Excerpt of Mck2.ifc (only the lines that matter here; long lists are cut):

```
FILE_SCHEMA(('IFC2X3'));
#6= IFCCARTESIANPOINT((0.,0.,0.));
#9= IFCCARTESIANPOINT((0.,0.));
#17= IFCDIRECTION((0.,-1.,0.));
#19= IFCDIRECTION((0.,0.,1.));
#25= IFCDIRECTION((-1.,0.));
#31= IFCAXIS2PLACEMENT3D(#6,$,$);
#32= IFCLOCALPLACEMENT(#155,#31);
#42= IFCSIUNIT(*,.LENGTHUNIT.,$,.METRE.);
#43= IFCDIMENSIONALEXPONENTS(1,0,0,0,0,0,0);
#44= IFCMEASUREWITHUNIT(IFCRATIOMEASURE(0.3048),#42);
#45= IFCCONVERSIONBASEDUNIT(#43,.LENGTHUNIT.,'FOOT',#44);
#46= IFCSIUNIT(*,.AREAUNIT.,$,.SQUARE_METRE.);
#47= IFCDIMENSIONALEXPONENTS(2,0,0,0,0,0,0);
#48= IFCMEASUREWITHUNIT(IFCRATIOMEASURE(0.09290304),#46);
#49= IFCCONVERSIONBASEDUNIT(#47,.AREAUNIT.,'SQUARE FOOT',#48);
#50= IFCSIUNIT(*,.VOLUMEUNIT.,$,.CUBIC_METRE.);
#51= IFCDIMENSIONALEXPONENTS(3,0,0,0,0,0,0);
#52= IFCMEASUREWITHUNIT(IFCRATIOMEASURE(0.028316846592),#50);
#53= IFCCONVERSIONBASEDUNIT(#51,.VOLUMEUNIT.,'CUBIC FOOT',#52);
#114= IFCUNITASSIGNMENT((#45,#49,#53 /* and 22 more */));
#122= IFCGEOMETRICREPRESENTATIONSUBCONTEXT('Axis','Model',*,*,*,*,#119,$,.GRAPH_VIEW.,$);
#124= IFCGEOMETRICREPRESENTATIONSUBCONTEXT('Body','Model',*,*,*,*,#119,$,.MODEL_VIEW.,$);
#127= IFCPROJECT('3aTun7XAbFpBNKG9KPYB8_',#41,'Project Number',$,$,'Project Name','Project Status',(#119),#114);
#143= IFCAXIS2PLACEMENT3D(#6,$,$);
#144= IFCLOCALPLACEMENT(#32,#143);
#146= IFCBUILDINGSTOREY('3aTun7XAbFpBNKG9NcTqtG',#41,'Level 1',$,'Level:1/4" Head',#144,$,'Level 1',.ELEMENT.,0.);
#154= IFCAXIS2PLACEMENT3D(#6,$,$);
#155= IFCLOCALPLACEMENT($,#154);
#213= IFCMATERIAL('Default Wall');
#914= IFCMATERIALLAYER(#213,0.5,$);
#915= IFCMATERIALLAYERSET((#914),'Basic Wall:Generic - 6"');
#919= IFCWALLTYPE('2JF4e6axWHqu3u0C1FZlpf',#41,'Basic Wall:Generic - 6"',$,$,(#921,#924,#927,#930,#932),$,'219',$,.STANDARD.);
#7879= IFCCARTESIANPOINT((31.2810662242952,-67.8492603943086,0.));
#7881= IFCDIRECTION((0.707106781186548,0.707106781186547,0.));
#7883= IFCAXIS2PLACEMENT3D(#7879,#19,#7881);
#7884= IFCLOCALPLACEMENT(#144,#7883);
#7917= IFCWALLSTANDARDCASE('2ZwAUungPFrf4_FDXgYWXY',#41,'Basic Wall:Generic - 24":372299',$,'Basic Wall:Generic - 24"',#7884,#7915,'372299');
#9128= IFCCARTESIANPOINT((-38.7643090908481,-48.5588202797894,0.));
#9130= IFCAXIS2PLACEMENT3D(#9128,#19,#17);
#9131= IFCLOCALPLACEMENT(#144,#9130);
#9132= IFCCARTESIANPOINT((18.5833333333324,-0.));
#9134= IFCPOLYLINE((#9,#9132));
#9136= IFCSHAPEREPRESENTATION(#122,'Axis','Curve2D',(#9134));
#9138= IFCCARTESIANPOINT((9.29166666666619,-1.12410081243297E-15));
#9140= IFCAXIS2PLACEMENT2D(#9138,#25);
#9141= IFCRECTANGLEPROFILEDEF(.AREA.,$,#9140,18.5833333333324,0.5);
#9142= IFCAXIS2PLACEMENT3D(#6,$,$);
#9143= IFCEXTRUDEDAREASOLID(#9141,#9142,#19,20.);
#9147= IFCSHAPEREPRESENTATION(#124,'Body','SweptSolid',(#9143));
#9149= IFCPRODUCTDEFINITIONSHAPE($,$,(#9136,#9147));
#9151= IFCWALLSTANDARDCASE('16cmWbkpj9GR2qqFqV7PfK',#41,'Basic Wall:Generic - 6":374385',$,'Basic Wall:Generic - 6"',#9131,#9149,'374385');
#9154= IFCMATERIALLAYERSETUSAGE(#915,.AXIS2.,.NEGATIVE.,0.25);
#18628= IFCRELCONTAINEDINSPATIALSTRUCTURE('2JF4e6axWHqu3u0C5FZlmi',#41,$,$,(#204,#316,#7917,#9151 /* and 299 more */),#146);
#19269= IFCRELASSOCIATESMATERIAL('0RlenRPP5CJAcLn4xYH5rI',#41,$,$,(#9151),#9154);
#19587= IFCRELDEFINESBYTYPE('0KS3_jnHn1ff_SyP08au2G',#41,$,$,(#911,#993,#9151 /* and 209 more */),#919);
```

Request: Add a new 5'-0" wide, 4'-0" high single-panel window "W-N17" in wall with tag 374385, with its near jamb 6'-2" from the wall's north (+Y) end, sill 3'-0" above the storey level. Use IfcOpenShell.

```python
import numpy as np
import ifcopenshell
import ifcopenshell.api.feature
import ifcopenshell.api.geometry
import ifcopenshell.api.root
import ifcopenshell.api.spatial
import ifcopenshell.api.type
import ifcopenshell.geom
import ifcopenshell.util.element
import ifcopenshell.util.placement
import ifcopenshell.util.representation
import ifcopenshell.util.shape
import ifcopenshell.util.unit

model = ifcopenshell.open("Mck2.ifc")
unit_scale = ifcopenshell.util.unit.calculate_unit_scale(model)
settings = ifcopenshell.geom.settings()


def volume(element):
    """Net volume in cubic metres, openings subtracted."""
    shape = ifcopenshell.geom.create_shape(settings, element)
    return ifcopenshell.util.shape.get_volume(shape.geometry)


wall = model.by_guid("16cmWbkpj9GR2qqFqV7PfK")
storey = ifcopenshell.util.element.get_container(wall, ifc_class="IfcBuildingStorey")
context = ifcopenshell.util.representation.get_context(model, "Model", "Body", "MODEL_VIEW")
before = volume(wall)

width, height, from_end, sill = 1.524, 1.2192, 1.8796, 0.9144  # metres

# The wall runs along its own X axis, and the end named is its -X end.
wall_shape = ifcopenshell.geom.create_shape(settings, wall)
x, y, z = ifcopenshell.util.shape.get_vertices(wall_shape.geometry).T
start = x.min() + from_end
face, thickness = float(y.min()), float(y.max() - y.min())
wall_matrix = ifcopenshell.util.placement.get_local_placement(wall.ObjectPlacement)
level = ifcopenshell.util.placement.get_local_placement(storey.ObjectPlacement)[2, 3]


def in_wall(x, y):
    """Placement at x, y metres in the wall's axes, at sill height."""
    matrix = wall_matrix.copy()
    matrix[:, 3] = wall_matrix @ np.array([x / unit_scale, y / unit_scale, 0.0, 1.0])
    matrix[2, 3] = level + sill / unit_scale
    return matrix


# Opening: a box that overshoots both wall faces by 50 mm.
opening = ifcopenshell.api.root.create_entity(model, ifc_class="IfcOpeningElement")
box = ifcopenshell.api.geometry.add_wall_representation(
    model, context=context, length=width, height=height, thickness=thickness + 0.1
)
ifcopenshell.api.geometry.assign_representation(model, product=opening, representation=box)
ifcopenshell.api.geometry.edit_object_placement(model, product=opening, matrix=in_wall(start, face - 0.05), is_si=False)
ifcopenshell.api.feature.add_feature(model, feature=opening, element=wall)

window = ifcopenshell.api.root.create_entity(model, ifc_class="IfcWindow", name="W-N17")
window.OverallWidth, window.OverallHeight = width / unit_scale, height / unit_scale
body = ifcopenshell.api.geometry.add_window_representation(
    model,
    context=context,
    overall_width=window.OverallWidth,
    overall_height=window.OverallHeight,
    partition_type="SINGLE_PANEL",
)
ifcopenshell.api.geometry.assign_representation(model, product=window, representation=body)
ifcopenshell.api.spatial.assign_container(model, products=[window], relating_structure=storey)
fills = ifcopenshell.api.feature.add_filling(model, opening=opening, element=window)
fills.OwnerHistory = window.OwnerHistory  # required in IFC2X3

# IFC2X3 keeps the operation on the window style.
style = ifcopenshell.api.root.create_entity(model, ifc_class="IfcWindowStyle", name="W-N17")
style.OperationType, style.ConstructionType = "SINGLE_PANEL", "NOTDEFINED"
style.ParameterTakesPrecedence = style.Sizeable = False
ifcopenshell.api.type.assign_type(model, related_objects=[window], relating_type=style)

# Centre the window in the wall's thickness.
ifcopenshell.api.geometry.edit_object_placement(model, product=window, matrix=in_wall(start, face), is_si=False)
window_shape = ifcopenshell.geom.create_shape(settings, window)
depth = ifcopenshell.util.shape.get_vertices(window_shape.geometry)[:, 1]
offset = face + thickness / 2 - (depth.min() + depth.max()) / 2
ifcopenshell.api.geometry.edit_object_placement(model, product=window, matrix=in_wall(start, offset), is_si=False)

after = volume(wall)

print(f"wall volume {before:.3f} -> {after:.3f} m3")

model.write("Mck2_edited.ifc")
```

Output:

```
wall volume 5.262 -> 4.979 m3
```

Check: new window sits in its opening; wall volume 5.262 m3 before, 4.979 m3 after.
